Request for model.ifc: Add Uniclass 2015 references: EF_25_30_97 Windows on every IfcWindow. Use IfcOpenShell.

First a look at what the model holds.

```python
import ifcopenshell

model = ifcopenshell.open("model.ifc")
print(model.schema)
print("classifications:", [c.Name for c in model.by_type("IfcClassification")])
for ifc_class in ("IfcDoor", "IfcRoof", "IfcStair", "IfcWall", "IfcWindow"):
    print(ifc_class, len(model.by_type(ifc_class)))
```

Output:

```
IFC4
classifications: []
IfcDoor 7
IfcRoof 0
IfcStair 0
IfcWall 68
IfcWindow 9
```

```python
import ifcopenshell
import ifcopenshell.api.classification

model = ifcopenshell.open("model.ifc")

system = ifcopenshell.api.classification.add_classification(model, classification="Uniclass 2015")

codes = {
    "IfcWindow": ("EF_25_30_97", "Windows"),
}
for ifc_class, (code, name) in codes.items():
    products = model.by_type(ifc_class)
    ifcopenshell.api.classification.add_reference(
        model, products=products, classification=system, identification=code, name=name
    )
    print(code, len(products))

model.write("model-out.ifc")
```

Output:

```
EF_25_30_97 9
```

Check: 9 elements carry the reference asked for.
